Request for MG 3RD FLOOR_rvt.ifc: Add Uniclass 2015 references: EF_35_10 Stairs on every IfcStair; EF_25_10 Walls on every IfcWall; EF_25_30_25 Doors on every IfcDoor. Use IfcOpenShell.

First a look at what the model holds.

```python
import ifcopenshell

model = ifcopenshell.open("MG 3RD FLOOR_rvt.ifc")
print(model.schema)
print("classifications:", [c.Name for c in model.by_type("IfcClassification")])
for ifc_class in ("IfcDoor", "IfcRoof", "IfcStair", "IfcWall", "IfcWindow"):
    print(ifc_class, len(model.by_type(ifc_class)))
```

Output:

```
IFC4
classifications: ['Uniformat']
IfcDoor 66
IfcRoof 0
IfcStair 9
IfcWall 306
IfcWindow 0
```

```python
import ifcopenshell
import ifcopenshell.api.classification

model = ifcopenshell.open("MG 3RD FLOOR_rvt.ifc")

system = ifcopenshell.api.classification.add_classification(model, classification="Uniclass 2015")

codes = {
    "IfcStair": ("EF_35_10", "Stairs"),
    "IfcWall": ("EF_25_10", "Walls"),
    "IfcDoor": ("EF_25_30_25", "Doors"),
}
for ifc_class, (code, name) in codes.items():
    products = model.by_type(ifc_class)
    ifcopenshell.api.classification.add_reference(
        model, products=products, classification=system, identification=code, name=name
    )
    print(code, len(products))

model.write("MG 3RD FLOOR_rvt_rev.ifc")
```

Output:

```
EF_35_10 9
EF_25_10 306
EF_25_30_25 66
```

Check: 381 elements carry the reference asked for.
